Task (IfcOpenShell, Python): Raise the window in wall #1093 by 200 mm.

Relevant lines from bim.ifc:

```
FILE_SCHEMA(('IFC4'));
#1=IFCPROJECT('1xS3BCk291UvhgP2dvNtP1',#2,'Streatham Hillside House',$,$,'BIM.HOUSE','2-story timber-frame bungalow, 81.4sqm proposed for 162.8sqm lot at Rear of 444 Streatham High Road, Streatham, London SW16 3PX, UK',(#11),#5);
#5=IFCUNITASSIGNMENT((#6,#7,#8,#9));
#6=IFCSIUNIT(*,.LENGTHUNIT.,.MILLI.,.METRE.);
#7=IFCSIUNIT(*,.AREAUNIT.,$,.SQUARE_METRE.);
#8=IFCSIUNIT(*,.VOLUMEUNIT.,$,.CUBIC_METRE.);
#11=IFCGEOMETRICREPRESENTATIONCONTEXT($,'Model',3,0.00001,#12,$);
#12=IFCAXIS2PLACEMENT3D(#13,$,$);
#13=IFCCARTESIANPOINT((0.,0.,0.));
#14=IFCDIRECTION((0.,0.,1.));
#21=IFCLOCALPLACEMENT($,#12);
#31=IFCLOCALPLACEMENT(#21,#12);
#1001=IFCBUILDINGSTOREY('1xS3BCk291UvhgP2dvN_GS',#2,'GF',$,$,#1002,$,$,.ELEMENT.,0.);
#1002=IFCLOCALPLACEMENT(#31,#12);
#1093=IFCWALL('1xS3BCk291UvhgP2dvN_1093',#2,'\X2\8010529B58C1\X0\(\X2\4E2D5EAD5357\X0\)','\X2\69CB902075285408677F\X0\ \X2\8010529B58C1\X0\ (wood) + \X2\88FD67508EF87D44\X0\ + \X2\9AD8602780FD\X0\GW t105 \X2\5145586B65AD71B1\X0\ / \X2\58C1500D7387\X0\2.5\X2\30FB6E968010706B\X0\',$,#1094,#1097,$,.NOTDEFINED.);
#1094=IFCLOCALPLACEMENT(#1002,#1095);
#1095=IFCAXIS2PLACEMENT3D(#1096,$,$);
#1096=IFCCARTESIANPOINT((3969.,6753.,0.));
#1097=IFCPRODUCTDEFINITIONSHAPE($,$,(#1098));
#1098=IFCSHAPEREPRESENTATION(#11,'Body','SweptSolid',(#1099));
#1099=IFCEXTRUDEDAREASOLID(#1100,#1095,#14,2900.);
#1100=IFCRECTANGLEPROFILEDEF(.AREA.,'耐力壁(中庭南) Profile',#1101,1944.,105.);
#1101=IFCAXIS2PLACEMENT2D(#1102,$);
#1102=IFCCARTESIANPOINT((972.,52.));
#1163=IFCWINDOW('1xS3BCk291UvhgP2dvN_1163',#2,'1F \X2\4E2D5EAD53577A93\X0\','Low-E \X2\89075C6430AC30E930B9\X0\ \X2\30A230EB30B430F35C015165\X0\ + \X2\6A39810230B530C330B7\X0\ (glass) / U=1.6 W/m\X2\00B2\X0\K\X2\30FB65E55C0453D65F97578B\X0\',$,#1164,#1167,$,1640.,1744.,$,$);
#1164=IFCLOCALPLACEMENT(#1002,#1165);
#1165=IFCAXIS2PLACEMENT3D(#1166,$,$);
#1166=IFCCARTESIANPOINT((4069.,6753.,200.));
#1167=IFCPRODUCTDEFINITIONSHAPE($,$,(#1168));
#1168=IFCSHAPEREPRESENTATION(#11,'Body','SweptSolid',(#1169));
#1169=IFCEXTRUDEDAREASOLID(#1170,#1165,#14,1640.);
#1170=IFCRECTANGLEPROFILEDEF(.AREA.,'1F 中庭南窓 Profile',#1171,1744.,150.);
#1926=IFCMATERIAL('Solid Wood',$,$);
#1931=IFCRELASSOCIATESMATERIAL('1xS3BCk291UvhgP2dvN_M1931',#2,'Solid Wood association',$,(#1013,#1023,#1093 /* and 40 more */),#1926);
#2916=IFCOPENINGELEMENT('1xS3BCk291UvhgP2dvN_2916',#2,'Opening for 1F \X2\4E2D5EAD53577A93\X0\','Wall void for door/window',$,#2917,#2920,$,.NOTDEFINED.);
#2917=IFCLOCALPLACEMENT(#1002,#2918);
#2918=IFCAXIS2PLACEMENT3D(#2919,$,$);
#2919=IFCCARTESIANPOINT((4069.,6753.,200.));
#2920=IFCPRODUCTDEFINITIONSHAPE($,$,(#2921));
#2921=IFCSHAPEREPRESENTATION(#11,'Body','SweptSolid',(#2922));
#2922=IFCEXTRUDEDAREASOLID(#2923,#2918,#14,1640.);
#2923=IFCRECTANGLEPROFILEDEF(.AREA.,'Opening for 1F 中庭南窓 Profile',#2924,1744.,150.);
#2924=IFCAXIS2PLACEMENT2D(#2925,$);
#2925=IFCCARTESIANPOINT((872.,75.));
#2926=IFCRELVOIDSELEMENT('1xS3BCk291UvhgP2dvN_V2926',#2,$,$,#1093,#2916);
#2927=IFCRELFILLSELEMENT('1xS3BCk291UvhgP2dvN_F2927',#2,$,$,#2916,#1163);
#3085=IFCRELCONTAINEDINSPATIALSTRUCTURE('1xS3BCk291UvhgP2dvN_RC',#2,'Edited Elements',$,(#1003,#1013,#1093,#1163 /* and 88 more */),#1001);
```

```python
import numpy as np
import ifcopenshell
import ifcopenshell.api.geometry
import ifcopenshell.util.placement
import ifcopenshell.util.unit

model = ifcopenshell.open("bim.ifc")
unit_scale = ifcopenshell.util.unit.calculate_unit_scale(model)

window = model.by_guid("1xS3BCk291UvhgP2dvN_1163")
opening = window.FillsVoids[0].RelatingOpeningElement
dz = 0.2 / unit_scale

shift = np.array([0.0, 0.0, dz])
# The window is not placed relative to its opening, so move both.
for product in (opening, window):
    matrix = ifcopenshell.util.placement.get_local_placement(product.ObjectPlacement)
    matrix[:3, 3] += shift
    ifcopenshell.api.geometry.edit_object_placement(model, product=product, matrix=matrix, is_si=False)

print(f"moved by {dz * unit_scale:+.3f} m")

model.write("bim_rev.ifc")
```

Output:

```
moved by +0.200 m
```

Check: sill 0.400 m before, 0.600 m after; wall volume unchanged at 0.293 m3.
